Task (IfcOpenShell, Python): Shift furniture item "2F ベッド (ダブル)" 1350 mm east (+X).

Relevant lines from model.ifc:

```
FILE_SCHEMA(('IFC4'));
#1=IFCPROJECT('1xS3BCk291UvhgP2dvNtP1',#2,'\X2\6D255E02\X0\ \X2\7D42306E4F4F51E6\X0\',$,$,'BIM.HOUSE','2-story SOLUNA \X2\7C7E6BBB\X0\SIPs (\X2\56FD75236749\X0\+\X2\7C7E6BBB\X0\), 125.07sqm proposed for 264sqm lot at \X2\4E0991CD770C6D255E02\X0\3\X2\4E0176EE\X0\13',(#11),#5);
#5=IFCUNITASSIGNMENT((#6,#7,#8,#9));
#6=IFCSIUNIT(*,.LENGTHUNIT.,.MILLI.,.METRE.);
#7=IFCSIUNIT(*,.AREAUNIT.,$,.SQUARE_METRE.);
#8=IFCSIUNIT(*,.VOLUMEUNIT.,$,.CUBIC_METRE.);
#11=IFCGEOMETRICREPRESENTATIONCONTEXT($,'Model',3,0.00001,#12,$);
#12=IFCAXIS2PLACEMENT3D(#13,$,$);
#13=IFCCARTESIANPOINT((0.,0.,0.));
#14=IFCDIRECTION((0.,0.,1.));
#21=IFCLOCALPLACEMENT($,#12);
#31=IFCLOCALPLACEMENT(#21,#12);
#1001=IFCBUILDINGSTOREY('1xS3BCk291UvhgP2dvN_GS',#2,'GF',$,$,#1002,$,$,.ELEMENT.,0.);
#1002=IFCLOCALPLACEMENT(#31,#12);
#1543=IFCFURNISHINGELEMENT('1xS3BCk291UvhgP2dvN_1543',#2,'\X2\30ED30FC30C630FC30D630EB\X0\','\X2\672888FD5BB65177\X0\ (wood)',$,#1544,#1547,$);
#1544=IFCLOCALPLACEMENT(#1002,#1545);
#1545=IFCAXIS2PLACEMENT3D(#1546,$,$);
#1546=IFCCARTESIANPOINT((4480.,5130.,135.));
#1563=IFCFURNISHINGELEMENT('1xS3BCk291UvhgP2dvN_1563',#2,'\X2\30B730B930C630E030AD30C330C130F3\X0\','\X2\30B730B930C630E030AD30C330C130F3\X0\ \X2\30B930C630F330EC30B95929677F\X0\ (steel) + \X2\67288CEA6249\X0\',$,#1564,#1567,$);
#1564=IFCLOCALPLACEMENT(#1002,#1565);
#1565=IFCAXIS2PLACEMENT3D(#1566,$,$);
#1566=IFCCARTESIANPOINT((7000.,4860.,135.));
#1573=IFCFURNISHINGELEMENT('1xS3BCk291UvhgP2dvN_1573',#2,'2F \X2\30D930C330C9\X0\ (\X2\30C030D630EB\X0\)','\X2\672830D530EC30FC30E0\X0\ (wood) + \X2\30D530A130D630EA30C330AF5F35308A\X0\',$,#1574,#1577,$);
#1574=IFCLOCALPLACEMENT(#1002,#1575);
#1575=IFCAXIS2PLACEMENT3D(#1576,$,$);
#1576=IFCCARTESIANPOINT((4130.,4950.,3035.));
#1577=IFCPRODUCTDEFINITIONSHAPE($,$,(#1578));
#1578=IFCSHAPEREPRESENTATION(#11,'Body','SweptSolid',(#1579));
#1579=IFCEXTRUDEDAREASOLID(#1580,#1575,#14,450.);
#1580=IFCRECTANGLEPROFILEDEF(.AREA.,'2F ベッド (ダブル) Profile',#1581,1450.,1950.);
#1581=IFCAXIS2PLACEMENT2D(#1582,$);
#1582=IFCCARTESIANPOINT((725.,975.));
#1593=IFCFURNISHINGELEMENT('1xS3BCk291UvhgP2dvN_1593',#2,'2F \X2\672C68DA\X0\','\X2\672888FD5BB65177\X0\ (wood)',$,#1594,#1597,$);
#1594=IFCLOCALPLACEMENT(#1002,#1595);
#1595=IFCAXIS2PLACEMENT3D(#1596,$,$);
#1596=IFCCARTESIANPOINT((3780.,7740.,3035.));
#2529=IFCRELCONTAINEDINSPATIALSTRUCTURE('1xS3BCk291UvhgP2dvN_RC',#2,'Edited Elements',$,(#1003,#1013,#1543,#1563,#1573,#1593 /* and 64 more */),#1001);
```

```python
import ifcopenshell
import ifcopenshell.api.geometry
import ifcopenshell.util.placement
import ifcopenshell.util.unit

model = ifcopenshell.open("model.ifc")
unit_scale = ifcopenshell.util.unit.calculate_unit_scale(model)

item = model.by_guid("1xS3BCk291UvhgP2dvN_1573")
matrix = ifcopenshell.util.placement.get_local_placement(item.ObjectPlacement)
matrix[0, 3] += 1.35 / unit_scale
ifcopenshell.api.geometry.edit_object_placement(model, product=item, matrix=matrix, is_si=False)

print(ifcopenshell.util.placement.get_local_placement(item.ObjectPlacement).round(3) + 0.0)

model.write("model_rev.ifc")
```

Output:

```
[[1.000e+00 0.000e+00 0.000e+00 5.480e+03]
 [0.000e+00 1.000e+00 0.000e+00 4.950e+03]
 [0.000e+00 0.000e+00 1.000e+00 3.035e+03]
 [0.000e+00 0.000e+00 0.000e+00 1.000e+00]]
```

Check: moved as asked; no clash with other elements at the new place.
